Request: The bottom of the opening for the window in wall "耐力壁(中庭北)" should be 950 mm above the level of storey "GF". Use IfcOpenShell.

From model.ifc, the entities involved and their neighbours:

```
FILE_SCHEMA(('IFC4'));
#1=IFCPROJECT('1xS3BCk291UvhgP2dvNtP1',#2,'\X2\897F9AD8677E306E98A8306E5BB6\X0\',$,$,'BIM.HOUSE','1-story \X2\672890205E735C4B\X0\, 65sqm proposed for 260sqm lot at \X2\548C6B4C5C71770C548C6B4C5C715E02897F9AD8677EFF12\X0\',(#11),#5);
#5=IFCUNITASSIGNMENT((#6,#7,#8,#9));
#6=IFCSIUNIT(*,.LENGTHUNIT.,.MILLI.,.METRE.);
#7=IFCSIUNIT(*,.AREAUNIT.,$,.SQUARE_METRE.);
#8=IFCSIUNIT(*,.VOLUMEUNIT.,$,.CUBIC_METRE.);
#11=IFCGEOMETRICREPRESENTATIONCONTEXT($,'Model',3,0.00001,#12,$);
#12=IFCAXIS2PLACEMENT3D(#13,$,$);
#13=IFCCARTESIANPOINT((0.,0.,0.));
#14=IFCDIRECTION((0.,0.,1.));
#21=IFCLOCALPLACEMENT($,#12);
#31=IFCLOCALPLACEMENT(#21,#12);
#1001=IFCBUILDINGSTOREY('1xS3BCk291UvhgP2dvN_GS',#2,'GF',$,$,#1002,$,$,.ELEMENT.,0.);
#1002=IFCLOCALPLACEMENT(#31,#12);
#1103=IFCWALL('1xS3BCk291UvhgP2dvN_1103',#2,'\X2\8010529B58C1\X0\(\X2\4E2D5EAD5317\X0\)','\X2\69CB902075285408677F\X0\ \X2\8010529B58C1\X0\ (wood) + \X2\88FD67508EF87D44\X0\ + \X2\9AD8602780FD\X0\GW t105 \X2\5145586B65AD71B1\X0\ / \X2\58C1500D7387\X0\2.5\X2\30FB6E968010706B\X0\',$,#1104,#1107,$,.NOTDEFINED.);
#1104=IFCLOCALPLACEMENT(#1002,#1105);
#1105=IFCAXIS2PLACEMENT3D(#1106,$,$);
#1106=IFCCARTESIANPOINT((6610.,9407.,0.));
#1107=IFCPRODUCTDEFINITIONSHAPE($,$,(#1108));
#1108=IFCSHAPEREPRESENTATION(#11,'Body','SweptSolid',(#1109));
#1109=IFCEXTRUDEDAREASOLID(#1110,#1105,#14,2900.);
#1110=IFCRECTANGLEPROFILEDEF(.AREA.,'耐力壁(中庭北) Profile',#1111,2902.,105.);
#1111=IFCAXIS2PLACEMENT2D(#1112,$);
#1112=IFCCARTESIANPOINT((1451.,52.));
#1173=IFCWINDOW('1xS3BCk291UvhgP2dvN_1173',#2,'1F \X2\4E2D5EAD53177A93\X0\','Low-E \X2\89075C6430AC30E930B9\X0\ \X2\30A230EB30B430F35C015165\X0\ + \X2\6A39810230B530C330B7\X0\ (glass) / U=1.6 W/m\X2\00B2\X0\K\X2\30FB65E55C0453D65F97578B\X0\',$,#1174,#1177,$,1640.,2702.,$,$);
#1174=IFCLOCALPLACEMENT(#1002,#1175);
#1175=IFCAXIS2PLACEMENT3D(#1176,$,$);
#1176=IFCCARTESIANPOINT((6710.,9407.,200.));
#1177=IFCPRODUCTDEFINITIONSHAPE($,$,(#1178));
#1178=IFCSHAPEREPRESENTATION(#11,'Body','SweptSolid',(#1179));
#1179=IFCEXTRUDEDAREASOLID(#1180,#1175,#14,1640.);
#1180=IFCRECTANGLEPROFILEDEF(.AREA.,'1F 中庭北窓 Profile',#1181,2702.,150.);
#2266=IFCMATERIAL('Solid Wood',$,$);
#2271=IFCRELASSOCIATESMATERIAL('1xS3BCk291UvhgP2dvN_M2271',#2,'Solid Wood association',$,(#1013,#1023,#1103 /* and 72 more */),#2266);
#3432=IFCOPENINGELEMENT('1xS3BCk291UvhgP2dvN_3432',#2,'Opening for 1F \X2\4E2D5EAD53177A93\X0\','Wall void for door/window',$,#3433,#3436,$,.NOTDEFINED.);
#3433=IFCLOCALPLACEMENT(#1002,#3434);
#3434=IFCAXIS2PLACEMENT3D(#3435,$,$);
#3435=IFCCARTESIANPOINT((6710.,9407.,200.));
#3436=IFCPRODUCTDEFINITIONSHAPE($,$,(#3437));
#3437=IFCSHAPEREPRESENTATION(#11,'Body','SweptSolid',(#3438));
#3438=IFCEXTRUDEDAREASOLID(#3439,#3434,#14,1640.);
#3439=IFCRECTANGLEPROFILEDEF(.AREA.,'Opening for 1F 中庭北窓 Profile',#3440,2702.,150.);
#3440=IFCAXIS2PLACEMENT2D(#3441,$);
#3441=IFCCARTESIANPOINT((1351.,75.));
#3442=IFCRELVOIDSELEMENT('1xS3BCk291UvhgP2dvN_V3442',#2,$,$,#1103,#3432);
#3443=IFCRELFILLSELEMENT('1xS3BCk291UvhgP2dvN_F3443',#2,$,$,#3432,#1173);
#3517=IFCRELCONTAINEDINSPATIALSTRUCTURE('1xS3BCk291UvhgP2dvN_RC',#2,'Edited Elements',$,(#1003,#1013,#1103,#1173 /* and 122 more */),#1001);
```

```python
import numpy as np
import ifcopenshell
import ifcopenshell.api.geometry
import ifcopenshell.geom
import ifcopenshell.util.element
import ifcopenshell.util.placement
import ifcopenshell.util.shape
import ifcopenshell.util.unit

model = ifcopenshell.open("model.ifc")
unit_scale = ifcopenshell.util.unit.calculate_unit_scale(model)

window = model.by_id(1173)
opening = window.FillsVoids[0].RelatingOpeningElement
storey = ifcopenshell.util.element.get_container(window, ifc_class="IfcBuildingStorey")
level = ifcopenshell.util.placement.get_local_placement(storey.ObjectPlacement)[2, 3]

# The opening's origin need not be at the sill, so measure its lowest point.
shape = ifcopenshell.geom.create_shape(ifcopenshell.geom.settings(), opening)
bottom = ifcopenshell.util.shape.get_shape_bottom_elevation(shape, shape.geometry) / unit_scale
dz = level + 0.95 / unit_scale - bottom

shift = np.array([0.0, 0.0, dz])
# The window is not placed relative to its opening, so move both.
for product in (opening, window):
    matrix = ifcopenshell.util.placement.get_local_placement(product.ObjectPlacement)
    matrix[:3, 3] += shift
    ifcopenshell.api.geometry.edit_object_placement(model, product=product, matrix=matrix, is_si=False)

print(f"moved by {dz * unit_scale:+.3f} m")

model.write("model_v2.ifc")
```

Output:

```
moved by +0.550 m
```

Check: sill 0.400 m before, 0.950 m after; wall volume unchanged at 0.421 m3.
